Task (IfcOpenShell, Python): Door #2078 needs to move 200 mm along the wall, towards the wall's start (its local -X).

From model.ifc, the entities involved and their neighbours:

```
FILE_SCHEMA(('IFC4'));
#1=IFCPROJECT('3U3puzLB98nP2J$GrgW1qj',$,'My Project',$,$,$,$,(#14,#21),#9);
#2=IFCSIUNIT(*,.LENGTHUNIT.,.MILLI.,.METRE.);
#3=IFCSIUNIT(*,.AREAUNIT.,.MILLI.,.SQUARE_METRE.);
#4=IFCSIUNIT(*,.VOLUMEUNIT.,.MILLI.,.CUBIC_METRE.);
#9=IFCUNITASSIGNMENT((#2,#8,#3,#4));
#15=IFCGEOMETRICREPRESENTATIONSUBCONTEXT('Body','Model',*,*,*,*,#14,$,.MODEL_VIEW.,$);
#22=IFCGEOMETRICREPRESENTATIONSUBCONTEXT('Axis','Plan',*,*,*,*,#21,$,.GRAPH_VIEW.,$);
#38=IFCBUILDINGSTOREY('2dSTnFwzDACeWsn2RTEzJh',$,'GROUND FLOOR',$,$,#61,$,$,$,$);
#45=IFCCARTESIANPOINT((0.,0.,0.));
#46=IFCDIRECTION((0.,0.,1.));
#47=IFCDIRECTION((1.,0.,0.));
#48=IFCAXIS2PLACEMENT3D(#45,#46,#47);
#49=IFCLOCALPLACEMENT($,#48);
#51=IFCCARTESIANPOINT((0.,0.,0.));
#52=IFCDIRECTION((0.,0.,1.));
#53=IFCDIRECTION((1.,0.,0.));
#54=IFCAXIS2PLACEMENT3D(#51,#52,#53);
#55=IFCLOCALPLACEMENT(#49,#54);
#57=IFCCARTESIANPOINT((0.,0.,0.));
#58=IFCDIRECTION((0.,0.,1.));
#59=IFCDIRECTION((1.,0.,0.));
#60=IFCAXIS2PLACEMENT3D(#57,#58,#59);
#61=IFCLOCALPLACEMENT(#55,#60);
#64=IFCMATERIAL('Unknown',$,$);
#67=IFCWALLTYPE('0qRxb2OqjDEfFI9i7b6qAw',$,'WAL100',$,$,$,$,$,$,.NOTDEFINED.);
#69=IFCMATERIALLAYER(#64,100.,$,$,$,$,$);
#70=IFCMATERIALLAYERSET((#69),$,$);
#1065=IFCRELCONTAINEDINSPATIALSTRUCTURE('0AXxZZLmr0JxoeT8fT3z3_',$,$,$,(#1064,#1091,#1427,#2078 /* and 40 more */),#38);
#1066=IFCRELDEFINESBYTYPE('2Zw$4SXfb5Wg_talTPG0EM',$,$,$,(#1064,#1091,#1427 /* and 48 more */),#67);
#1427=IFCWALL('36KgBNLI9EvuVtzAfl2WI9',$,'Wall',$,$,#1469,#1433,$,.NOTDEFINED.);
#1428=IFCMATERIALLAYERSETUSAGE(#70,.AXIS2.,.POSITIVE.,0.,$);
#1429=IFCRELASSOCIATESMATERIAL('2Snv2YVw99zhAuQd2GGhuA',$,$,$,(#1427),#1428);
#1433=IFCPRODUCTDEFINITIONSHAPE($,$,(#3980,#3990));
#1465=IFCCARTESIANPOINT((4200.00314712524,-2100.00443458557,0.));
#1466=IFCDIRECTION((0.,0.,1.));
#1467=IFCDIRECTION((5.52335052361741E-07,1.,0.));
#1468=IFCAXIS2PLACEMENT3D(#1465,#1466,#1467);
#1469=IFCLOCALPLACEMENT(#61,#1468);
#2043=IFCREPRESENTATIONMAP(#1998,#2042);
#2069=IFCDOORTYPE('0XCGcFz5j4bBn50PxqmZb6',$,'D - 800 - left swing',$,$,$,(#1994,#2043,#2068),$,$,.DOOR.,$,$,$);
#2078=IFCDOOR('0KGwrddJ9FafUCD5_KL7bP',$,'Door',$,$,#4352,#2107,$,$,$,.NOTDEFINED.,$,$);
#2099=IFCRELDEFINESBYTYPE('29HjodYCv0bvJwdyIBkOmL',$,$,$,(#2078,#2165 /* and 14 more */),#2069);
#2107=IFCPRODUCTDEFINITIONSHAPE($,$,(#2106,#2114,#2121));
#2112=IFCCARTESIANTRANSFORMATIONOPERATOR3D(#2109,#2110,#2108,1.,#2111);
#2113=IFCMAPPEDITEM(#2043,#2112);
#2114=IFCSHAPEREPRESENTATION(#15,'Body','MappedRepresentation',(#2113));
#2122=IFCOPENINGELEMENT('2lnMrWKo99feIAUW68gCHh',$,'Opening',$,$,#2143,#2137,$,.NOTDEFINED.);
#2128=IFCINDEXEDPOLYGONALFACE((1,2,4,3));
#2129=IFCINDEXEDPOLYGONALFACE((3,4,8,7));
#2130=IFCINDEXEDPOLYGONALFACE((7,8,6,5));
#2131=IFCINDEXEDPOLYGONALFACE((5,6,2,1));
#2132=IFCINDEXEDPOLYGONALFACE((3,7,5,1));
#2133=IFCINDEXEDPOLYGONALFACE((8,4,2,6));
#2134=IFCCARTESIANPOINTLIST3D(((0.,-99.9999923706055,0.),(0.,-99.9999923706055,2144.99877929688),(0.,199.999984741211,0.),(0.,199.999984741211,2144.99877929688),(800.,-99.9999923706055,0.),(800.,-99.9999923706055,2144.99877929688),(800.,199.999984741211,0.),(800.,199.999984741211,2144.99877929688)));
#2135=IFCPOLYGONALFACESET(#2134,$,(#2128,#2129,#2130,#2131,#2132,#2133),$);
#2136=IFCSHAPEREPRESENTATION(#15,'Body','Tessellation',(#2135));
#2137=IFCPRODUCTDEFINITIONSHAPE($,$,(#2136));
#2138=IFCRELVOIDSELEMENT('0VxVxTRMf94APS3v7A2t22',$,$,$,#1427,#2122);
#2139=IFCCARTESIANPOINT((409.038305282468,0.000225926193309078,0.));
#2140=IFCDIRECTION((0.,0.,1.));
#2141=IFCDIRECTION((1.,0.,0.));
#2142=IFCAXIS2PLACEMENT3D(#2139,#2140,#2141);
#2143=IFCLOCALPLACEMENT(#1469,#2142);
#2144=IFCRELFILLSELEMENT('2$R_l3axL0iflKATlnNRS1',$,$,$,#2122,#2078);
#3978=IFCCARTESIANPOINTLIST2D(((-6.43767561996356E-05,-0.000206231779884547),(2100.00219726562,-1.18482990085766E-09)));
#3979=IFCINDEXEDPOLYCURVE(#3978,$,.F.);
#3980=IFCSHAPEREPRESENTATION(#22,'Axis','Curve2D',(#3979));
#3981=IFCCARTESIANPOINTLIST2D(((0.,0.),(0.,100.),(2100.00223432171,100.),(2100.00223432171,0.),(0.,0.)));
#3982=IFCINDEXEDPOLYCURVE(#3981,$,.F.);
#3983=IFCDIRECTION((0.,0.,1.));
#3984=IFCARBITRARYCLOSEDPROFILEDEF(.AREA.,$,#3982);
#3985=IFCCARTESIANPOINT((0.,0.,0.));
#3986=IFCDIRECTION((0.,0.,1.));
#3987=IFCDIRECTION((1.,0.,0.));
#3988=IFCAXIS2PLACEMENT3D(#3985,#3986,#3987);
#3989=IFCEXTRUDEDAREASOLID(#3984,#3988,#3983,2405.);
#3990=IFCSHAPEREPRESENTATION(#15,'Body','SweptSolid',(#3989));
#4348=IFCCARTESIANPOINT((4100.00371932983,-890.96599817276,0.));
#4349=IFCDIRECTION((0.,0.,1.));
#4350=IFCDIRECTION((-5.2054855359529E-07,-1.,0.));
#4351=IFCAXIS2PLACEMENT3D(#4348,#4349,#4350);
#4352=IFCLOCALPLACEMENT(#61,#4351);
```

```python
import ifcopenshell
import ifcopenshell.api.geometry
import ifcopenshell.util.placement
import ifcopenshell.util.unit

model = ifcopenshell.open("model.ifc")
unit_scale = ifcopenshell.util.unit.calculate_unit_scale(model)

door = model.by_guid("0KGwrddJ9FafUCD5_KL7bP")
opening = door.FillsVoids[0].RelatingOpeningElement
wall = opening.VoidsElements[0].RelatingBuildingElement

wall_matrix = ifcopenshell.util.placement.get_local_placement(wall.ObjectPlacement)
shift = wall_matrix[:3, 0] * -0.2 / unit_scale
before = ifcopenshell.util.placement.get_local_placement(door.ObjectPlacement)[:3, 3].copy()

# The door is not placed relative to its opening, so move both.
for product in (opening, door):
    matrix = ifcopenshell.util.placement.get_local_placement(product.ObjectPlacement)
    matrix[:3, 3] += shift
    ifcopenshell.api.geometry.edit_object_placement(model, product=product, matrix=matrix, is_si=False)

after = ifcopenshell.util.placement.get_local_placement(door.ObjectPlacement)[:3, 3]
print("door moved by", (after - before).round(3) + 0.0)

model.write("model_edited.ifc")
```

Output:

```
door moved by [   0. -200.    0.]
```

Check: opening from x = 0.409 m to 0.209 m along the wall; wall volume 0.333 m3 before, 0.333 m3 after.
